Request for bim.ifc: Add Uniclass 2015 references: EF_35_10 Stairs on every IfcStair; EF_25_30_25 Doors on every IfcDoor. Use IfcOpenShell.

First a look at what the model holds.

```python
import ifcopenshell

model = ifcopenshell.open("bim.ifc")
print(model.schema)
print("classifications:", [c.Name for c in model.by_type("IfcClassification")])
for ifc_class in ("IfcDoor", "IfcRoof", "IfcStair", "IfcWall", "IfcWindow"):
    print(ifc_class, len(model.by_type(ifc_class)))
```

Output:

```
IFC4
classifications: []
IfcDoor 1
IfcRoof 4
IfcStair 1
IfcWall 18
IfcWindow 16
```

```python
import ifcopenshell
import ifcopenshell.api.classification

model = ifcopenshell.open("bim.ifc")

system = ifcopenshell.api.classification.add_classification(model, classification="Uniclass 2015")

codes = {
    "IfcStair": ("EF_35_10", "Stairs"),
    "IfcDoor": ("EF_25_30_25", "Doors"),
}
for ifc_class, (code, name) in codes.items():
    products = model.by_type(ifc_class)
    ifcopenshell.api.classification.add_reference(
        model, products=products, classification=system, identification=code, name=name
    )
    print(code, len(products))

model.write("bim_edited.ifc")
```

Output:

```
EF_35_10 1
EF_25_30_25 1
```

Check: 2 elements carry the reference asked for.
